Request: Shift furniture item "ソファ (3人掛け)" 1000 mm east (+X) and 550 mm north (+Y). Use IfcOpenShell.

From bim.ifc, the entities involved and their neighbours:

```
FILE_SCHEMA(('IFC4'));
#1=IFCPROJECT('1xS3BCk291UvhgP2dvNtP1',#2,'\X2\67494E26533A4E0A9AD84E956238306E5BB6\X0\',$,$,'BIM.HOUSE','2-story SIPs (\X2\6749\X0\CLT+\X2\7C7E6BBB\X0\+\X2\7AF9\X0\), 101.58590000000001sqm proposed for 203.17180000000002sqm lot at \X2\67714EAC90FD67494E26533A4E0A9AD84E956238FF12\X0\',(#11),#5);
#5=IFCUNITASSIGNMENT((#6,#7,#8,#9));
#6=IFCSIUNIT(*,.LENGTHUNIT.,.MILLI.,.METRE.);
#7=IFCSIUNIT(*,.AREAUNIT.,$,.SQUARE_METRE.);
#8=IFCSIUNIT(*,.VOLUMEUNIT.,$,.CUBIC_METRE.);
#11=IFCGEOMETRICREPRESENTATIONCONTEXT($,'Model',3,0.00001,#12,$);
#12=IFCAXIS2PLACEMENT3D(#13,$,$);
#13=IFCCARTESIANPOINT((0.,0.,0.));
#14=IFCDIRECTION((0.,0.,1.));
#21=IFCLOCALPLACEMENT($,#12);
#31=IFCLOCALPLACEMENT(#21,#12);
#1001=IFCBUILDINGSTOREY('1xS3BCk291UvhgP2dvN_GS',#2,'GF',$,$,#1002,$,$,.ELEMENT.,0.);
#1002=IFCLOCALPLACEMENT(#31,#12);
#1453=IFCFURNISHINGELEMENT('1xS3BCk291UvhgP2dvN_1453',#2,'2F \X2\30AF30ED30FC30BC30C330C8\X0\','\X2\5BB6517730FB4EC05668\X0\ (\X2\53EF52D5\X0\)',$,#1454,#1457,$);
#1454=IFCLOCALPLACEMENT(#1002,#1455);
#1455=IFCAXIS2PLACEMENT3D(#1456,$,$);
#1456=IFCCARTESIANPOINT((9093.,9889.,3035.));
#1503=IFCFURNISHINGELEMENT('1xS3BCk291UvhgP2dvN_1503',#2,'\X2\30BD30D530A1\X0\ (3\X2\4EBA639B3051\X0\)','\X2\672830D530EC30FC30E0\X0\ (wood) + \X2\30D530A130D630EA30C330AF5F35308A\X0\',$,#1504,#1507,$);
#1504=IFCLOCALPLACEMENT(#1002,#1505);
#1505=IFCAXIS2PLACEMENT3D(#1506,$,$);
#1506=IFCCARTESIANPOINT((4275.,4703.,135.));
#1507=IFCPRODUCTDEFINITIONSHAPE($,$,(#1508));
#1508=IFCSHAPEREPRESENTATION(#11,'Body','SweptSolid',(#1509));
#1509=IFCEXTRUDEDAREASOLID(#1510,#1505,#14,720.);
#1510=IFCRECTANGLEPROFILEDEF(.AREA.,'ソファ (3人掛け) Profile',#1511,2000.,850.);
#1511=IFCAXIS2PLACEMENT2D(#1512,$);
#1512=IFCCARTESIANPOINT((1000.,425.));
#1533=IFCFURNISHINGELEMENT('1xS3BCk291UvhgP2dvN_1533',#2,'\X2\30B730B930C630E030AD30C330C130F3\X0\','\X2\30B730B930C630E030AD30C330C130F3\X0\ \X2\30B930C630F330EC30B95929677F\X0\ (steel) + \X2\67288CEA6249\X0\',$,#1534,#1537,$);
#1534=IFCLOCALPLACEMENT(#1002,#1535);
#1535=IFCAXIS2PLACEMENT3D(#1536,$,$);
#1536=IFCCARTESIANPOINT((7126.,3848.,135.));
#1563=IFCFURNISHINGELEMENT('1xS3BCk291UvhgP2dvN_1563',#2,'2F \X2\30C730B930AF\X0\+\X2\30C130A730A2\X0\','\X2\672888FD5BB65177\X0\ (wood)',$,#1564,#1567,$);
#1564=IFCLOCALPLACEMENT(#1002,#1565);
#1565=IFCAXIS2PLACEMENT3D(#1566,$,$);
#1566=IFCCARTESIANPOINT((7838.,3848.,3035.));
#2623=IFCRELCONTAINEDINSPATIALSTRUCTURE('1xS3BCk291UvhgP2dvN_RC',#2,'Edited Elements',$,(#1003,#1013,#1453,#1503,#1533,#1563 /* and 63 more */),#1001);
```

```python
import ifcopenshell
import ifcopenshell.api.geometry
import ifcopenshell.util.placement

model = ifcopenshell.open("bim.ifc")

item = model.by_id(1503)
matrix = ifcopenshell.util.placement.get_local_placement(item.ObjectPlacement)
matrix[0, 3] += 1000.0
matrix[1, 3] += 550.0
ifcopenshell.api.geometry.edit_object_placement(model, product=item, matrix=matrix, is_si=False)

print(ifcopenshell.util.placement.get_local_placement(item.ObjectPlacement).round(3) + 0.0)

model.write("bim_edited.ifc")
```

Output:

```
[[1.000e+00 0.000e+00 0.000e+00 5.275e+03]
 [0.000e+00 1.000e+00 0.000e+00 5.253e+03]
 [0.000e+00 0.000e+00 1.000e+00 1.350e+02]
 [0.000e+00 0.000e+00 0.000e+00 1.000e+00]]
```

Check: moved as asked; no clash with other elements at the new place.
